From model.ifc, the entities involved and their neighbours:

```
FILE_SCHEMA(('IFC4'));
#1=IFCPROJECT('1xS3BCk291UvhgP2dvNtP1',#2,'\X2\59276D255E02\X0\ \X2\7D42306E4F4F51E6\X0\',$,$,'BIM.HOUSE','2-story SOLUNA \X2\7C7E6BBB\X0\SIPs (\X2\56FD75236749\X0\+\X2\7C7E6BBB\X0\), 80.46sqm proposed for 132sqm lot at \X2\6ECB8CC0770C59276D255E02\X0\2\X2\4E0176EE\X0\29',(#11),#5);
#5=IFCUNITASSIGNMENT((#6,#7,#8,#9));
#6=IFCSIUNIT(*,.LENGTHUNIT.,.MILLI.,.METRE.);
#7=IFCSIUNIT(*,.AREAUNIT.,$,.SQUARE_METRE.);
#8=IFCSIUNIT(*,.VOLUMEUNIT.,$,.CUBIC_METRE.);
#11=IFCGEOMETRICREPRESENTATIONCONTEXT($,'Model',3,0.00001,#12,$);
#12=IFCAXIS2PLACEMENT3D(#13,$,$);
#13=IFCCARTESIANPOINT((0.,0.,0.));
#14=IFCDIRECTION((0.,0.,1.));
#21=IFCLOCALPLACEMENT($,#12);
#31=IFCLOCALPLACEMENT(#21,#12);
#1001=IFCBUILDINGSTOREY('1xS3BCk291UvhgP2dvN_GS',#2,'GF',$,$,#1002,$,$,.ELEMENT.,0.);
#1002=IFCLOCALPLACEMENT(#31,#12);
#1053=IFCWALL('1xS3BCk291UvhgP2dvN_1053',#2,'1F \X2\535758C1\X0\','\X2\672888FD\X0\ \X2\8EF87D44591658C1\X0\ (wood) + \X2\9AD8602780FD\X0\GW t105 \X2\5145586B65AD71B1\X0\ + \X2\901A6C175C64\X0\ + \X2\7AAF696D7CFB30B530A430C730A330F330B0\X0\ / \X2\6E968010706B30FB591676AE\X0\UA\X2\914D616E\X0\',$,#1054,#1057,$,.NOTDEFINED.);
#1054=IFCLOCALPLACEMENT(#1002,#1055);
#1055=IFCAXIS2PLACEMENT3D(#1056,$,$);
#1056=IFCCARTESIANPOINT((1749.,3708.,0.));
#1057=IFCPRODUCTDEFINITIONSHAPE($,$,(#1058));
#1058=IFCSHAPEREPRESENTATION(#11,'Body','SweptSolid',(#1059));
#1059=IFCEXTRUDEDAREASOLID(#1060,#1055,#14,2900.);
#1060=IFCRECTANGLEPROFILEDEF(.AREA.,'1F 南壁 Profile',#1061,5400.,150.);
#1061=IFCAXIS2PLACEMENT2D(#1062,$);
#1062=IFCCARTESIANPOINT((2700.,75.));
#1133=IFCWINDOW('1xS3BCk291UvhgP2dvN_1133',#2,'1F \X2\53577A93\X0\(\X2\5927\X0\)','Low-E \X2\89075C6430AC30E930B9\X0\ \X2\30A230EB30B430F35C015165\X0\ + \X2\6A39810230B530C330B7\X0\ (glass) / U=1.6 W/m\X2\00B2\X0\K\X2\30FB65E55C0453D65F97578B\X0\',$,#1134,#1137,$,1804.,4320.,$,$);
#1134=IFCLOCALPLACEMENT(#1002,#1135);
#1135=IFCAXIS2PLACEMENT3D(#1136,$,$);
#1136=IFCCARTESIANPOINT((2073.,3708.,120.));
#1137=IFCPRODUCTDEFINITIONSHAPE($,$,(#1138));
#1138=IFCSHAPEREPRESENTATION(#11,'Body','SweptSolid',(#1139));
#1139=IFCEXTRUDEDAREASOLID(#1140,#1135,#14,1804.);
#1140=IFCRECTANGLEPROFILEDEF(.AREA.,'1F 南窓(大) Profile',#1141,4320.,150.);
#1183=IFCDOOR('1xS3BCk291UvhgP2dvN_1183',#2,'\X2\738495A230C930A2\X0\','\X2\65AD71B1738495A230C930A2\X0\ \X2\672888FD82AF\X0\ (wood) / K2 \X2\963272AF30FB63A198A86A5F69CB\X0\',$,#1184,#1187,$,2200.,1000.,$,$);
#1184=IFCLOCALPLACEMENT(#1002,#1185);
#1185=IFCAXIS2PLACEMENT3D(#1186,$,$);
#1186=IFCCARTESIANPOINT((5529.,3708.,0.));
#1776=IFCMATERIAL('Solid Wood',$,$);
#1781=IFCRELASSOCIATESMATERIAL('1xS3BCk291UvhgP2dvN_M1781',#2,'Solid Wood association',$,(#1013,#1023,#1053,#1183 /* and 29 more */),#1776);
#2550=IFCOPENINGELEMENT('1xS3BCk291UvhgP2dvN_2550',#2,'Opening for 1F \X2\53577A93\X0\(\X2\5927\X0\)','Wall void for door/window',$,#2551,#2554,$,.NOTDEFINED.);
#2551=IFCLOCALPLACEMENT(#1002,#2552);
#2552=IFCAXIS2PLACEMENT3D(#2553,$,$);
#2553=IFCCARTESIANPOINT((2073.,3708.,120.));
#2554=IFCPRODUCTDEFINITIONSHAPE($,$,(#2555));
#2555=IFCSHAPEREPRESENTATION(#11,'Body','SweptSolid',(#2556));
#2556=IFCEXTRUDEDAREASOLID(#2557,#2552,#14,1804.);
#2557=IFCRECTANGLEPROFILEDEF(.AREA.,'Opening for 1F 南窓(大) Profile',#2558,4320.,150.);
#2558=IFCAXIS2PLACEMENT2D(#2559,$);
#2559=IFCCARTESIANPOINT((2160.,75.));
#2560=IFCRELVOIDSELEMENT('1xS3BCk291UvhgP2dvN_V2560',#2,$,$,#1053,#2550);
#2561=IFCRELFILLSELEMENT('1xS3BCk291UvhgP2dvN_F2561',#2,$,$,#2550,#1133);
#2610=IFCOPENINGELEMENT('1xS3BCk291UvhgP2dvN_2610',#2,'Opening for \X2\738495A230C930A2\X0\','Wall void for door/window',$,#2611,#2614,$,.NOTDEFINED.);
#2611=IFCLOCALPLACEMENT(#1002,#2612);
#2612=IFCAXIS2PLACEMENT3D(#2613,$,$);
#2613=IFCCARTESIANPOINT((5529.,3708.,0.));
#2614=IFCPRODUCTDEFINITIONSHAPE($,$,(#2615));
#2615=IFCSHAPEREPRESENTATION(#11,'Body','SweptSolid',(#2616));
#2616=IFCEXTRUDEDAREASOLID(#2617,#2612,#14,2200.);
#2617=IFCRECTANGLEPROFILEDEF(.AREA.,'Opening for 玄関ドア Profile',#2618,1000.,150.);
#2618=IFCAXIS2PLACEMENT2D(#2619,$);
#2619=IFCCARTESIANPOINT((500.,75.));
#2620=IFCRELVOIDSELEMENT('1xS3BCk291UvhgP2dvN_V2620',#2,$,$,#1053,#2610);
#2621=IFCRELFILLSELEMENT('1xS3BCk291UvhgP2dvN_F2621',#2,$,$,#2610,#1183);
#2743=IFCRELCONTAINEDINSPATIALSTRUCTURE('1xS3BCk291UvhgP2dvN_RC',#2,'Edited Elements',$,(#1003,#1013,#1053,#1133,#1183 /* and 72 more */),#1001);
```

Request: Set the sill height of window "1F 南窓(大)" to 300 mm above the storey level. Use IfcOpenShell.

```python
import numpy as np
import ifcopenshell
import ifcopenshell.api.geometry
import ifcopenshell.geom
import ifcopenshell.util.element
import ifcopenshell.util.placement
import ifcopenshell.util.shape
import ifcopenshell.util.unit

model = ifcopenshell.open("model.ifc")
unit_scale = ifcopenshell.util.unit.calculate_unit_scale(model)

window = model.by_id(1133)
opening = window.FillsVoids[0].RelatingOpeningElement
storey = ifcopenshell.util.element.get_container(window, ifc_class="IfcBuildingStorey")
level = ifcopenshell.util.placement.get_local_placement(storey.ObjectPlacement)[2, 3]

# The opening's origin need not be at the sill, so measure its lowest point.
shape = ifcopenshell.geom.create_shape(ifcopenshell.geom.settings(), opening)
bottom = ifcopenshell.util.shape.get_shape_bottom_elevation(shape, shape.geometry) / unit_scale
dz = level + 0.3 / unit_scale - bottom

shift = np.array([0.0, 0.0, dz])
# The window is not placed relative to its opening, so move both.
for product in (opening, window):
    matrix = ifcopenshell.util.placement.get_local_placement(product.ObjectPlacement)
    matrix[:3, 3] += shift
    ifcopenshell.api.geometry.edit_object_placement(model, product=product, matrix=matrix, is_si=False)

print(f"moved by {dz * unit_scale:+.3f} m")

model.write("model_updated.ifc")
```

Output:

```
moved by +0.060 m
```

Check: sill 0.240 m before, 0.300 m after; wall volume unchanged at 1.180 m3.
